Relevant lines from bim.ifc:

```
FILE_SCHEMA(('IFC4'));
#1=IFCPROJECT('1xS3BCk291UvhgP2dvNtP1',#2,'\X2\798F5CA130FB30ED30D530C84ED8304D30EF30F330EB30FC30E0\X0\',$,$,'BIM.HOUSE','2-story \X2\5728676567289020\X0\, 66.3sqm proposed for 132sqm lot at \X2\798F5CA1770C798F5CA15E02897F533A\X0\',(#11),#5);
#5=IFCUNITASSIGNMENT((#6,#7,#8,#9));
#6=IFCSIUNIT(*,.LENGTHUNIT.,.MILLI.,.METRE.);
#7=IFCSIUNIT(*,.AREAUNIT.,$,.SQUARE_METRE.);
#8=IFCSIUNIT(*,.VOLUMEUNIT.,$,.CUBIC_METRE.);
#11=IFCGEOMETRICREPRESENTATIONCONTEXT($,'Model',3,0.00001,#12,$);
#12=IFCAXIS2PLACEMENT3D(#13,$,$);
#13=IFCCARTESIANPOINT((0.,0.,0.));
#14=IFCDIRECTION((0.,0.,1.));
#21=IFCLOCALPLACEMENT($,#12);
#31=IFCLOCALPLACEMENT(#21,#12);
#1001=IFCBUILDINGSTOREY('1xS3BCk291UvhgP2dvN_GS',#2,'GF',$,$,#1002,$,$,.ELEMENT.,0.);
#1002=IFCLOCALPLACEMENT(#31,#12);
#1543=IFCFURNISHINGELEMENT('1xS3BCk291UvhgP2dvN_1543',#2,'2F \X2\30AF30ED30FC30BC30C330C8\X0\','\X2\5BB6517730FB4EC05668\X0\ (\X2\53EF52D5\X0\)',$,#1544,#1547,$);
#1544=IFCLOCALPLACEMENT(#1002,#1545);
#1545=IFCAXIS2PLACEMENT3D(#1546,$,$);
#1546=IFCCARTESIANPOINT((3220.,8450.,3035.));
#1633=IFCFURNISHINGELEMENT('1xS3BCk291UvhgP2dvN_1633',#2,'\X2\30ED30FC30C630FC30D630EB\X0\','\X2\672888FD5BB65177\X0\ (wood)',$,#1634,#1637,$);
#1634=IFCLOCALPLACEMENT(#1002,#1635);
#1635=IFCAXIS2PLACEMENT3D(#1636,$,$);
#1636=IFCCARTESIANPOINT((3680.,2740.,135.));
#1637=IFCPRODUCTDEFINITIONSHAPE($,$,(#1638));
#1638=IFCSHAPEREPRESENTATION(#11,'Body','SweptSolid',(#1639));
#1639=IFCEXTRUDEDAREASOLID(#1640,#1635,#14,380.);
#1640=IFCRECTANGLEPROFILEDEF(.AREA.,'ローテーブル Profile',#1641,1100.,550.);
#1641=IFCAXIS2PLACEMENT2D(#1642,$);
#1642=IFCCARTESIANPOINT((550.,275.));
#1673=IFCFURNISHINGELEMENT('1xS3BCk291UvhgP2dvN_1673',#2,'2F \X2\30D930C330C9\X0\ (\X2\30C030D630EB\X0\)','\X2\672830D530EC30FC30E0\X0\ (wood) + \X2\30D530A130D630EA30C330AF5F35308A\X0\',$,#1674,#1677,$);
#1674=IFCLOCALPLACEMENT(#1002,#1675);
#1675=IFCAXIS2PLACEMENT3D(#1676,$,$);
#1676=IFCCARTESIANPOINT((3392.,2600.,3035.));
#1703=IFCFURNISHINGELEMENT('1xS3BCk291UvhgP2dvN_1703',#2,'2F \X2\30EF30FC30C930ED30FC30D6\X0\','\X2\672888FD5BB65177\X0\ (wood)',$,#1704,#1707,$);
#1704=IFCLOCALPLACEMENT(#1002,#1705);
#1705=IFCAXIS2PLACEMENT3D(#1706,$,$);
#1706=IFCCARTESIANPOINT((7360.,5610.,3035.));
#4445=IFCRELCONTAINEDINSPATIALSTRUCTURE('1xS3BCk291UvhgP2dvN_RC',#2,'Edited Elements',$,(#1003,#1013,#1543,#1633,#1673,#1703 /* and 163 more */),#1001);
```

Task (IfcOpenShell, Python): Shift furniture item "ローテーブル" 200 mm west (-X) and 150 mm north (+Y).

```python
import ifcopenshell
import ifcopenshell.api.geometry
import ifcopenshell.util.placement
import ifcopenshell.util.unit

model = ifcopenshell.open("bim.ifc")
unit_scale = ifcopenshell.util.unit.calculate_unit_scale(model)

item = model.by_guid("1xS3BCk291UvhgP2dvN_1633")
matrix = ifcopenshell.util.placement.get_local_placement(item.ObjectPlacement)
matrix[0, 3] -= 0.2 / unit_scale
matrix[1, 3] += 0.15 / unit_scale
ifcopenshell.api.geometry.edit_object_placement(model, product=item, matrix=matrix, is_si=False)

print(ifcopenshell.util.placement.get_local_placement(item.ObjectPlacement).round(3) + 0.0)

model.write("bim_rev.ifc")
```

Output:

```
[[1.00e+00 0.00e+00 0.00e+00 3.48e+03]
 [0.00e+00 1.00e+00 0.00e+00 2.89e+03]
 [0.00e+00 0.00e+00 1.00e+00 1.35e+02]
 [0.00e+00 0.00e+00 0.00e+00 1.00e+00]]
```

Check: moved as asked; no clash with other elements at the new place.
